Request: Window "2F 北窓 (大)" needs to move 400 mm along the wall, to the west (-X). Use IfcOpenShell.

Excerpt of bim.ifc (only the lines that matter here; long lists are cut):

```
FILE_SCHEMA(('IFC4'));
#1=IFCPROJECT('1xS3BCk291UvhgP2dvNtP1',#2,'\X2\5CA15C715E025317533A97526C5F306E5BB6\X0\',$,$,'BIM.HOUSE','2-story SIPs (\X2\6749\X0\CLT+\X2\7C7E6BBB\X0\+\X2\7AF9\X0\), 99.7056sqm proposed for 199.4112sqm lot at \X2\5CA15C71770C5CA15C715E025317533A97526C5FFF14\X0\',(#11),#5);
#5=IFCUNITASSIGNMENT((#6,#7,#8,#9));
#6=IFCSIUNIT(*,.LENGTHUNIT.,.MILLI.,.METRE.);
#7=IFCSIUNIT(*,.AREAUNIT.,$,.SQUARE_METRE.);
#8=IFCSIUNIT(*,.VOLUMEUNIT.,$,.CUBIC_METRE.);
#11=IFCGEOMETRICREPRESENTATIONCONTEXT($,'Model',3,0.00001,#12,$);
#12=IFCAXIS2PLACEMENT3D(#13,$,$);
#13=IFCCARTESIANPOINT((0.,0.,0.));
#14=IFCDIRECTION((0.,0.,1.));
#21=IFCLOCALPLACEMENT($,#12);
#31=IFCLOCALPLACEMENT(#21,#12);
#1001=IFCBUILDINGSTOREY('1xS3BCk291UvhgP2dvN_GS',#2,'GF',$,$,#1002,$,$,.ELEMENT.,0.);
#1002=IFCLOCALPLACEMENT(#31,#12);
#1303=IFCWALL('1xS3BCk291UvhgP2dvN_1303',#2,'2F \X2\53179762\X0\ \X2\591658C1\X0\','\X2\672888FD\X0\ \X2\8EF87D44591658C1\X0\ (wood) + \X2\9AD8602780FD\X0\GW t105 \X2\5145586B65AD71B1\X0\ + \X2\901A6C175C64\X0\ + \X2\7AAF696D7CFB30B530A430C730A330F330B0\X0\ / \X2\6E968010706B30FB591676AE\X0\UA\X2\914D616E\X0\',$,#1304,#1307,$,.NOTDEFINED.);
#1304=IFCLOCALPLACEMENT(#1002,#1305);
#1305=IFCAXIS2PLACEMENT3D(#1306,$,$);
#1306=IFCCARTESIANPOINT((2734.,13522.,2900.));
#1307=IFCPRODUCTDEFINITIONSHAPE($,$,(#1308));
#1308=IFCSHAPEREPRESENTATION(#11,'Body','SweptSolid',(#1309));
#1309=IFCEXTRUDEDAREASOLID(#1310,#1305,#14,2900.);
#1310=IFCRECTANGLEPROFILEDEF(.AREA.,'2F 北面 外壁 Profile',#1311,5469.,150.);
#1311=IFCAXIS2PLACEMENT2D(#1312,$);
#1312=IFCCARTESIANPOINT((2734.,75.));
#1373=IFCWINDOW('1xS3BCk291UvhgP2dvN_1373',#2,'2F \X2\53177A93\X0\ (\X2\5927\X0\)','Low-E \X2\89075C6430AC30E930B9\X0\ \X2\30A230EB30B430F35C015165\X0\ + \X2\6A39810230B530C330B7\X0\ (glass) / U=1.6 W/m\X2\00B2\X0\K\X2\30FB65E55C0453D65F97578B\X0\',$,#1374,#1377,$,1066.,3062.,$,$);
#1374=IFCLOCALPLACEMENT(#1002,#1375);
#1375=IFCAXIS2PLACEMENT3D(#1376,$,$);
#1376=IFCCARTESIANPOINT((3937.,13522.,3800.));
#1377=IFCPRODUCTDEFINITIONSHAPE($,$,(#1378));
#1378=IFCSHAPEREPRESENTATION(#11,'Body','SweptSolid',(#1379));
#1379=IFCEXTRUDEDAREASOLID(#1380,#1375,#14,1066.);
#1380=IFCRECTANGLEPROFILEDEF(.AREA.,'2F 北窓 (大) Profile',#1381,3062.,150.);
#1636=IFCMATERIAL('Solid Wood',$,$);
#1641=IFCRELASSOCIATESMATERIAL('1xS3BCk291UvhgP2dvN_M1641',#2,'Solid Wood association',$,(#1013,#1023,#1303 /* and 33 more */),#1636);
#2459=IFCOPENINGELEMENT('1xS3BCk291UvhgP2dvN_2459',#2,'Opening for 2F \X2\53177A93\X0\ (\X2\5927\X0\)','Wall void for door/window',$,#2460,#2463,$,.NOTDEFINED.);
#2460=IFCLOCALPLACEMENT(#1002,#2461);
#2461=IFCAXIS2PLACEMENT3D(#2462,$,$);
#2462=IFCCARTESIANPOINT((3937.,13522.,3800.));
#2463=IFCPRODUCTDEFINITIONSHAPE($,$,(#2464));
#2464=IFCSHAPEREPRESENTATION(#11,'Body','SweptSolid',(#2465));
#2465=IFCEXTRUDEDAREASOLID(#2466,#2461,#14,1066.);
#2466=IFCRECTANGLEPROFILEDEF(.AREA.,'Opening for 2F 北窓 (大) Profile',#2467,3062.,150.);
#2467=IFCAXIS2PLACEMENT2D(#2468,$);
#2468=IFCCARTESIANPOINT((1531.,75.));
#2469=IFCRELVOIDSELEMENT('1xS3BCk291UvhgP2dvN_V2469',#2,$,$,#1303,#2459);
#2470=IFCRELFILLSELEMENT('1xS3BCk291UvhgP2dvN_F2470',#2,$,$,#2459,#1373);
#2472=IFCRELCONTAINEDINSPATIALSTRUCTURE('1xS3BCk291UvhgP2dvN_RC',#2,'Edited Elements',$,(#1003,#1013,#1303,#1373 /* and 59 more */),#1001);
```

```python
import ifcopenshell
import ifcopenshell.api.geometry
import ifcopenshell.util.placement
import ifcopenshell.util.unit

model = ifcopenshell.open("bim.ifc")
unit_scale = ifcopenshell.util.unit.calculate_unit_scale(model)

window = model.by_guid("1xS3BCk291UvhgP2dvN_1373")
opening = window.FillsVoids[0].RelatingOpeningElement
wall = opening.VoidsElements[0].RelatingBuildingElement

wall_matrix = ifcopenshell.util.placement.get_local_placement(wall.ObjectPlacement)
shift = wall_matrix[:3, 0] * -0.4 / unit_scale
before = ifcopenshell.util.placement.get_local_placement(window.ObjectPlacement)[:3, 3].copy()

# The window is not placed relative to its opening, so move both.
for product in (opening, window):
    matrix = ifcopenshell.util.placement.get_local_placement(product.ObjectPlacement)
    matrix[:3, 3] += shift
    ifcopenshell.api.geometry.edit_object_placement(model, product=product, matrix=matrix, is_si=False)

after = ifcopenshell.util.placement.get_local_placement(window.ObjectPlacement)[:3, 3]
print("window moved by", (after - before).round(3) + 0.0)

model.write("bim_v2.ifc")
```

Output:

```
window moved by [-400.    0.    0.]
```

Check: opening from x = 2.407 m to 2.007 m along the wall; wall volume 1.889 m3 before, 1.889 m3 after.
